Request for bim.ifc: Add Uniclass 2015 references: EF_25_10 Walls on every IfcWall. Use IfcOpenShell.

First a look at what the model holds.

```python
import ifcopenshell

model = ifcopenshell.open("bim.ifc")
print(model.schema)
print("classifications:", [c.Name for c in model.by_type("IfcClassification")])
for ifc_class in ("IfcDoor", "IfcRoof", "IfcStair", "IfcWall", "IfcWindow"):
    print(ifc_class, len(model.by_type(ifc_class)))
```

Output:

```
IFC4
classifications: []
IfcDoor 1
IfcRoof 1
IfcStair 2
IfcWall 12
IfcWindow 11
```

```python
import ifcopenshell
import ifcopenshell.api.classification

model = ifcopenshell.open("bim.ifc")

system = ifcopenshell.api.classification.add_classification(model, classification="Uniclass 2015")

codes = {
    "IfcWall": ("EF_25_10", "Walls"),
}
for ifc_class, (code, name) in codes.items():
    products = model.by_type(ifc_class)
    ifcopenshell.api.classification.add_reference(
        model, products=products, classification=system, identification=code, name=name
    )
    print(code, len(products))

model.write("bim_rev.ifc")
```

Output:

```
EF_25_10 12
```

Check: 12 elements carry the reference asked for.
